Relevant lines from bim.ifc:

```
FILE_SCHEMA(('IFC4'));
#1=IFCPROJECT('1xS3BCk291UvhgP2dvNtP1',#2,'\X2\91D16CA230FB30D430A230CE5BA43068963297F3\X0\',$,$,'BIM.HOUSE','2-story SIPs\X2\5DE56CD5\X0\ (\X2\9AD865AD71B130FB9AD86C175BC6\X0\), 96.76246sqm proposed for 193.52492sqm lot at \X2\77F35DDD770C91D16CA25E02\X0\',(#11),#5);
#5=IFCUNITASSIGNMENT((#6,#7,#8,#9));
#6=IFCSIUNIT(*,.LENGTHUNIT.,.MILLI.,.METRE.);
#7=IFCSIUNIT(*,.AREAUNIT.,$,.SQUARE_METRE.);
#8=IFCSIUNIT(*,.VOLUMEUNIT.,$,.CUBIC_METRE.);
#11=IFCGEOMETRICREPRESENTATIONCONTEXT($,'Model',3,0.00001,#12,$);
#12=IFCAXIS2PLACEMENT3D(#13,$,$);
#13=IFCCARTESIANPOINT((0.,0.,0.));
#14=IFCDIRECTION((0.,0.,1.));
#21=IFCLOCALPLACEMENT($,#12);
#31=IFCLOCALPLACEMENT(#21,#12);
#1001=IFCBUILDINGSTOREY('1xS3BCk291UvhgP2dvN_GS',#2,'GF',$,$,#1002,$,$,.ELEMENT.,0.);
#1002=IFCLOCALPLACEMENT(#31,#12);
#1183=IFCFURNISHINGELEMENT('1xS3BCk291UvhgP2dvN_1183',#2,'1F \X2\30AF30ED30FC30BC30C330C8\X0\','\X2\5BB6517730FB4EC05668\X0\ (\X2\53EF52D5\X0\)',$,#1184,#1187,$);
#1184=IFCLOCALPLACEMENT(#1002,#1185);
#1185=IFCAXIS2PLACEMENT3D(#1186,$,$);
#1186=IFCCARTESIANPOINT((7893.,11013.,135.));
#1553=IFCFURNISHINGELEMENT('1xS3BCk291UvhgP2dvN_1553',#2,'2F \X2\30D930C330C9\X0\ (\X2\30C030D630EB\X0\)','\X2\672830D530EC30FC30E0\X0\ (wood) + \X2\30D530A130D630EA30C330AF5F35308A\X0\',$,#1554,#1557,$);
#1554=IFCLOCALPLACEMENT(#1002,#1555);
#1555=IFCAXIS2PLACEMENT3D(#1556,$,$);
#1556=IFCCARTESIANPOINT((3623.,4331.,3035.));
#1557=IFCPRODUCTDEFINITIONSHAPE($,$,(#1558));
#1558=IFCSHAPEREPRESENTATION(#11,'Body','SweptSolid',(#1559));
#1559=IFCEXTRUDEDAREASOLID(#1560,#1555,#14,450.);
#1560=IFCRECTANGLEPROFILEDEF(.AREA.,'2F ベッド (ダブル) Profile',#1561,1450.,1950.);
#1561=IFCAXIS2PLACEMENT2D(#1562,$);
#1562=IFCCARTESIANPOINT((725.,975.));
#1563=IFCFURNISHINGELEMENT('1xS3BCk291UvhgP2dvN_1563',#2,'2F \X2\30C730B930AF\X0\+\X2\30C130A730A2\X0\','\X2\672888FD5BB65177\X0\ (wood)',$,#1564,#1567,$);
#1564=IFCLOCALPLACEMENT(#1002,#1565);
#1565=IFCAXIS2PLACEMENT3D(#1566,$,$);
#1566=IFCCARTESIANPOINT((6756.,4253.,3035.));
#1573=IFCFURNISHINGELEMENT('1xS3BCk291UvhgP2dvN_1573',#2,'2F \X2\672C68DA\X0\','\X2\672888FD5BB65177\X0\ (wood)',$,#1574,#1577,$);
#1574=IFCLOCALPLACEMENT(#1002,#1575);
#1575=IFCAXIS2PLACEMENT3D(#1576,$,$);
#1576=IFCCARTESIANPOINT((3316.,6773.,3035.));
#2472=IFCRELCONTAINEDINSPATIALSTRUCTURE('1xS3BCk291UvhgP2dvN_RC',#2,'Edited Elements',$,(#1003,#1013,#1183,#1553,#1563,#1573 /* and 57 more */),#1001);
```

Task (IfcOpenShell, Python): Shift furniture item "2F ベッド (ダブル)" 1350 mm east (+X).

```python
import ifcopenshell
import ifcopenshell.api.geometry
import ifcopenshell.util.placement

model = ifcopenshell.open("bim.ifc")

item = model.by_guid("1xS3BCk291UvhgP2dvN_1553")
matrix = ifcopenshell.util.placement.get_local_placement(item.ObjectPlacement)
matrix[0, 3] += 1350.0
ifcopenshell.api.geometry.edit_object_placement(model, product=item, matrix=matrix, is_si=False)

print(ifcopenshell.util.placement.get_local_placement(item.ObjectPlacement).round(3) + 0.0)

model.write("bim_v2.ifc")
```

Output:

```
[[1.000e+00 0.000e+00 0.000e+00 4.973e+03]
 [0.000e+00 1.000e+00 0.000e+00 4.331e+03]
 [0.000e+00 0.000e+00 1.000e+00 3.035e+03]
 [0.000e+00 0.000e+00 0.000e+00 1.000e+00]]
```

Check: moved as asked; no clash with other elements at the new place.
